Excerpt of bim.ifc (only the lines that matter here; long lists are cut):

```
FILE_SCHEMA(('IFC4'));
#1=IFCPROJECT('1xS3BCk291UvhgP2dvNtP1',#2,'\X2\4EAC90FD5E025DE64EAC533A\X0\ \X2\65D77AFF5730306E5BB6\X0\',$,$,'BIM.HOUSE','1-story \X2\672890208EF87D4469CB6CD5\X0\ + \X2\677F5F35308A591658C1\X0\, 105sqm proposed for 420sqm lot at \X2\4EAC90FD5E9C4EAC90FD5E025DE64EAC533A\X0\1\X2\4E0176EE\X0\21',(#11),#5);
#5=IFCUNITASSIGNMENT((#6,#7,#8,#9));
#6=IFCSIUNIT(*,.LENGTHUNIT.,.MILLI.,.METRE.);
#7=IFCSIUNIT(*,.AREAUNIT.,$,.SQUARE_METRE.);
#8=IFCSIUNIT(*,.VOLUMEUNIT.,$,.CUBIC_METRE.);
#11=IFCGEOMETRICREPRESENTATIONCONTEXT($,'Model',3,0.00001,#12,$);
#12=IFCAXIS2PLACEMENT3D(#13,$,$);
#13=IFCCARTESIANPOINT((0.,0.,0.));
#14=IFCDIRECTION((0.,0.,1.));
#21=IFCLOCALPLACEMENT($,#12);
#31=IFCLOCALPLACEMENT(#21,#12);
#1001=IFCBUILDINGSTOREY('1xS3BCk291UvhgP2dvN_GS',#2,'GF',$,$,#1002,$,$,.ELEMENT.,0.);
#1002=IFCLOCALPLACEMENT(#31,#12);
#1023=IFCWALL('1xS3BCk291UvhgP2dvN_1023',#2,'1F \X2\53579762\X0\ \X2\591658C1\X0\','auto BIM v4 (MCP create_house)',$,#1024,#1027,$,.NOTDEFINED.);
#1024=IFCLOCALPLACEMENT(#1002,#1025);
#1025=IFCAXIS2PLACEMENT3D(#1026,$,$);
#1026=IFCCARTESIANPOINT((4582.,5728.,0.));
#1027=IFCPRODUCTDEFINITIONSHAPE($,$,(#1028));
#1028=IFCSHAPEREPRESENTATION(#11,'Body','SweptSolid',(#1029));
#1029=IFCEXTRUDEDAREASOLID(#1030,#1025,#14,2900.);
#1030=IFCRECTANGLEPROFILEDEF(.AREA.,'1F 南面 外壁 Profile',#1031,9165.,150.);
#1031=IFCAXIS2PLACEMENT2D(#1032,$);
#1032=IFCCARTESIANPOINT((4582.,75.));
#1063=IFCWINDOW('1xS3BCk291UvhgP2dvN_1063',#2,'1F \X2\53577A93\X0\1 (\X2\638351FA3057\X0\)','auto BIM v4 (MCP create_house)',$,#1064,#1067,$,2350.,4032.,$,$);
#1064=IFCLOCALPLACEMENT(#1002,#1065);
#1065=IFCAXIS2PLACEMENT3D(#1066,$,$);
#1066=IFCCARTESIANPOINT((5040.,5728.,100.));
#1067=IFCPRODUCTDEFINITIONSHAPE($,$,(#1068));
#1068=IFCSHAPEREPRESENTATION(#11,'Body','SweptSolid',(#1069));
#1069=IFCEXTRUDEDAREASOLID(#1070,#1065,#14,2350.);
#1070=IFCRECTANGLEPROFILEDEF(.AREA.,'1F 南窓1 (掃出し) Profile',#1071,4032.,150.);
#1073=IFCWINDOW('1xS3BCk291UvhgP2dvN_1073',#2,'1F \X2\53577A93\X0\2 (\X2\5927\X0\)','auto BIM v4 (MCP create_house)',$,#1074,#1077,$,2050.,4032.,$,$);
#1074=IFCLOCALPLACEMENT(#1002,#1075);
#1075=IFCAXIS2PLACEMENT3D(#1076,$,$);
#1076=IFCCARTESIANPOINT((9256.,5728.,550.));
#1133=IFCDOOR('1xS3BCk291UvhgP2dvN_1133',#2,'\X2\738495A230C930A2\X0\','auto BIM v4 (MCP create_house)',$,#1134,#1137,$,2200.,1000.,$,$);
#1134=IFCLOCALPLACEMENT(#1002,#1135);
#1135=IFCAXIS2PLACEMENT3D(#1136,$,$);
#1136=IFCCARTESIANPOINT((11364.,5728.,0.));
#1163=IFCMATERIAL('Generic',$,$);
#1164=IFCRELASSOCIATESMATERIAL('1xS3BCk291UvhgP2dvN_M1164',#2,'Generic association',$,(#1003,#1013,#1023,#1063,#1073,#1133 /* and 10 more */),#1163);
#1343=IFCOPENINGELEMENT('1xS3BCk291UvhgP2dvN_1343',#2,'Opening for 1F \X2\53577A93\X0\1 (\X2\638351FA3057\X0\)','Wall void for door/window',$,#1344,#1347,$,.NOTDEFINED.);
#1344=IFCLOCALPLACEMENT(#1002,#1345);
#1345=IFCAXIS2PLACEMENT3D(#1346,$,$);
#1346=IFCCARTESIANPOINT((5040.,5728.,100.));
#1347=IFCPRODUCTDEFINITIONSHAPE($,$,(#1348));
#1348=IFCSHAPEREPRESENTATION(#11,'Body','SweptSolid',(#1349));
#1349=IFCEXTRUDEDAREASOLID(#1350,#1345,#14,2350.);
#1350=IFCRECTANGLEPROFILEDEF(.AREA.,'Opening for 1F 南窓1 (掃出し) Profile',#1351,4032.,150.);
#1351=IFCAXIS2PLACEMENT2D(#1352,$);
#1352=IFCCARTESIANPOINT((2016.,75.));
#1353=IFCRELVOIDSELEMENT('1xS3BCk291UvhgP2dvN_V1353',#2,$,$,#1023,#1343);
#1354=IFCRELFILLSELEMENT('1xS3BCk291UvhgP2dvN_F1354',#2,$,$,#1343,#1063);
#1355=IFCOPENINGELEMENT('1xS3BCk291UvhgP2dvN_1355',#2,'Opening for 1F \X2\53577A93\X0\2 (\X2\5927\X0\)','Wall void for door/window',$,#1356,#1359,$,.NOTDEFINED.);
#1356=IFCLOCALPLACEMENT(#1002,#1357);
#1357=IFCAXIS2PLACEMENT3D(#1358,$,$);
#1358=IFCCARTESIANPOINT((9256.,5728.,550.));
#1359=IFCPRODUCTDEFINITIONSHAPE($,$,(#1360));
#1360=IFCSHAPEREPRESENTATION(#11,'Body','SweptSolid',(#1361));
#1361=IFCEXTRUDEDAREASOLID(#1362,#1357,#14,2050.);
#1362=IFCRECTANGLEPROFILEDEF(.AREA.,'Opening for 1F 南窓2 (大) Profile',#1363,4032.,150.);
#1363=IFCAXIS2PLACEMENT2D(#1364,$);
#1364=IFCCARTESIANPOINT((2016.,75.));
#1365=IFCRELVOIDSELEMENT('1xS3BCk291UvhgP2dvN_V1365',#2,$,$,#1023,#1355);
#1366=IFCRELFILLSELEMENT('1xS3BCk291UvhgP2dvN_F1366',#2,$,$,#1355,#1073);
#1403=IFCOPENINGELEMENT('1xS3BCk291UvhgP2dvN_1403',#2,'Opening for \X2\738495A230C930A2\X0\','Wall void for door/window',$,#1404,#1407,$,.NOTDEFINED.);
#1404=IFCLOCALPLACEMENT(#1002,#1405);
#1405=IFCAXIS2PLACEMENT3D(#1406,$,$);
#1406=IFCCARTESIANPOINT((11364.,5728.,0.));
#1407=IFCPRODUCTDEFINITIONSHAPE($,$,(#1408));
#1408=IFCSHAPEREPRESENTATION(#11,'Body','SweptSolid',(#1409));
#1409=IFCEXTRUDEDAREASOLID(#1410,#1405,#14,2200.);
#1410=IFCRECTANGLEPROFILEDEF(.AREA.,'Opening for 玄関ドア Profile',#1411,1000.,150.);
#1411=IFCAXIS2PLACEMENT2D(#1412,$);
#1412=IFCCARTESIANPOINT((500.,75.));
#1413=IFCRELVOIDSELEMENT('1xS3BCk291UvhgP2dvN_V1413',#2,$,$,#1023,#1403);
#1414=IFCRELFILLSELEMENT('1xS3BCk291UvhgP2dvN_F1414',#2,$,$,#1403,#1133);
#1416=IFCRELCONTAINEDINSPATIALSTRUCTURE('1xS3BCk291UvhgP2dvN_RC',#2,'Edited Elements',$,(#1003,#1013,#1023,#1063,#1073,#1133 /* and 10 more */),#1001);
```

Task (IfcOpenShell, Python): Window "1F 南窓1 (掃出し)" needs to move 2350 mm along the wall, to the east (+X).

```python
import ifcopenshell
import ifcopenshell.api.geometry
import ifcopenshell.util.placement

model = ifcopenshell.open("bim.ifc")

window = model.by_guid("1xS3BCk291UvhgP2dvN_1063")
opening = window.FillsVoids[0].RelatingOpeningElement
wall = opening.VoidsElements[0].RelatingBuildingElement

wall_matrix = ifcopenshell.util.placement.get_local_placement(wall.ObjectPlacement)
shift = wall_matrix[:3, 0] * 2350.0
before = ifcopenshell.util.placement.get_local_placement(window.ObjectPlacement)[:3, 3].copy()

# The window is not placed relative to its opening, so move both.
for product in (opening, window):
    matrix = ifcopenshell.util.placement.get_local_placement(product.ObjectPlacement)
    matrix[:3, 3] += shift
    ifcopenshell.api.geometry.edit_object_placement(model, product=product, matrix=matrix, is_si=False)

after = ifcopenshell.util.placement.get_local_placement(window.ObjectPlacement)[:3, 3]
print("window moved by", (after - before).round(3) + 0.0)

model.write("bim_v2.ifc")
```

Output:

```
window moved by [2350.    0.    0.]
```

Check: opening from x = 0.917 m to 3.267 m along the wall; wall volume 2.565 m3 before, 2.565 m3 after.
